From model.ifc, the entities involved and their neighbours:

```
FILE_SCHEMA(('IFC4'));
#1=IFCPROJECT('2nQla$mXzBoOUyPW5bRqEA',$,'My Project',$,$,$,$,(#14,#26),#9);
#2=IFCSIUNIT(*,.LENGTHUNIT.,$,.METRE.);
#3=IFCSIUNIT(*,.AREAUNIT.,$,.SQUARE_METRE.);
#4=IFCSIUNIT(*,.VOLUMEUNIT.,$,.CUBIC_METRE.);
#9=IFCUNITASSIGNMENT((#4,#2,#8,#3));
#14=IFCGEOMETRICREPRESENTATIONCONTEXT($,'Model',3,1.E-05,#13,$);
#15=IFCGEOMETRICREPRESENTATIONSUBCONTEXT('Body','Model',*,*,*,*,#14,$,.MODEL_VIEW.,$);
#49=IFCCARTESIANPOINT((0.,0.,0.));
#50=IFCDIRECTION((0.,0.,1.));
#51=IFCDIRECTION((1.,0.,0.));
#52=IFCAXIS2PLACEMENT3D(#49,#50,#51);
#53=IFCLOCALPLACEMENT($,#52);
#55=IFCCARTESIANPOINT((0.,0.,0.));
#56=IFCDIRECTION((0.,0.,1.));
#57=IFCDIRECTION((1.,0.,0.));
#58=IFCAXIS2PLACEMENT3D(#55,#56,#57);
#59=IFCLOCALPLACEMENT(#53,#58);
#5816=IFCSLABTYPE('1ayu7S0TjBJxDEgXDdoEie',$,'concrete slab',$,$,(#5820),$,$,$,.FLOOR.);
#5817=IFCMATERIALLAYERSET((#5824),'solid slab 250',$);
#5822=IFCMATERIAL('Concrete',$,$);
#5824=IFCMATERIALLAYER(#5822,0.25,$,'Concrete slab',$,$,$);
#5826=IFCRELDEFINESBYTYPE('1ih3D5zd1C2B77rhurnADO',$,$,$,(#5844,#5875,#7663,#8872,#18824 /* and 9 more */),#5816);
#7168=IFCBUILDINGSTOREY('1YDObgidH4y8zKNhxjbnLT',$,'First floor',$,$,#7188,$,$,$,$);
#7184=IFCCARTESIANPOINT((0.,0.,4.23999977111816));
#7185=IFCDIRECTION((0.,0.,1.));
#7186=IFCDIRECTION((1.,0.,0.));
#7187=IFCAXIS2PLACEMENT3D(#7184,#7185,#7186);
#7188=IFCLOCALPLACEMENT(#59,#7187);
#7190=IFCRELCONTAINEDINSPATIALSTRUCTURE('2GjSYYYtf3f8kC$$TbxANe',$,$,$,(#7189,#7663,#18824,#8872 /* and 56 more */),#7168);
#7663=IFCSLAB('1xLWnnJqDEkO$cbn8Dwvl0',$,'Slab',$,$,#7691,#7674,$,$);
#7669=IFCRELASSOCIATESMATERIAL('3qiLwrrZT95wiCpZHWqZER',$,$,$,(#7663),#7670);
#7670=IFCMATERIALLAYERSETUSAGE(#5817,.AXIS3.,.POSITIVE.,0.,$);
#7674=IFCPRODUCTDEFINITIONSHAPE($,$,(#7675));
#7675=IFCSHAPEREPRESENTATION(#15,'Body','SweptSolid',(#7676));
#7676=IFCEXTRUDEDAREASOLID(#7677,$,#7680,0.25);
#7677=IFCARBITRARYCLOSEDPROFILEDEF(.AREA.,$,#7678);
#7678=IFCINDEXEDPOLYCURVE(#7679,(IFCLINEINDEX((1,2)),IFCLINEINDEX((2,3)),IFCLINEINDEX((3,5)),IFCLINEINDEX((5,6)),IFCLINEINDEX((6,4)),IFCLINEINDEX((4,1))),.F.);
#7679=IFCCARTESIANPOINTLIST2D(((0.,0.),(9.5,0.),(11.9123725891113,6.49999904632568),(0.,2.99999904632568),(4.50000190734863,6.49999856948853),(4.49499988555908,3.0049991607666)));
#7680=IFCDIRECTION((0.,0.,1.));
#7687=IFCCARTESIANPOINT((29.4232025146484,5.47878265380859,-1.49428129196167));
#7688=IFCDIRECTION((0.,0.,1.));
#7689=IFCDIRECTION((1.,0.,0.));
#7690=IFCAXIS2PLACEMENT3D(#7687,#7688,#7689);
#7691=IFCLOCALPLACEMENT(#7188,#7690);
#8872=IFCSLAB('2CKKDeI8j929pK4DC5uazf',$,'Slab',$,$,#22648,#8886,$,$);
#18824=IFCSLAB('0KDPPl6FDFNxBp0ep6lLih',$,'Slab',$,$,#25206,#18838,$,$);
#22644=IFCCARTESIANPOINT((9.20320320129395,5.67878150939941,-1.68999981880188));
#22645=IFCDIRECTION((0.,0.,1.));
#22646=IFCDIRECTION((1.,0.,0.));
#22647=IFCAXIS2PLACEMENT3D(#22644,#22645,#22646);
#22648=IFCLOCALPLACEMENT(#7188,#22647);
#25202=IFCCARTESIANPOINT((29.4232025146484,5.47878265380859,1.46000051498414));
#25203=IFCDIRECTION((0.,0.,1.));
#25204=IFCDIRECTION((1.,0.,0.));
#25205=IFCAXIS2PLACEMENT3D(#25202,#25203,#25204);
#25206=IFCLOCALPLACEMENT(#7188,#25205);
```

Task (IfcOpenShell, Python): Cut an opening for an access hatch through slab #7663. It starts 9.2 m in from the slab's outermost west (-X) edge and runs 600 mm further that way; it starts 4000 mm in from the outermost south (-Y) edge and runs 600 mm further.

```python
import numpy as np
import ifcopenshell
import ifcopenshell.api.feature
import ifcopenshell.api.geometry
import ifcopenshell.api.root
import ifcopenshell.geom
import ifcopenshell.util.placement
import ifcopenshell.util.representation
import ifcopenshell.util.shape
import ifcopenshell.util.unit

model = ifcopenshell.open("model.ifc")
unit_scale = ifcopenshell.util.unit.calculate_unit_scale(model)
settings = ifcopenshell.geom.settings()


def volume(element):
    """Net volume in cubic metres, openings subtracted."""
    shape = ifcopenshell.geom.create_shape(settings, element)
    return ifcopenshell.util.shape.get_volume(shape.geometry)


slab = model.by_guid("1xLWnnJqDEkO$cbn8Dwvl0")
before = volume(slab)

# Extent in the slab's own axes, in metres. The edges named are its -X and -Y sides.
slab_shape = ifcopenshell.geom.create_shape(settings, slab)
vertices = ifcopenshell.util.shape.get_vertices(slab_shape.geometry)
x_min, y_min, bottom = vertices.min(axis=0)
top = vertices[:, 2].max()

opening = ifcopenshell.api.root.create_entity(model, ifc_class="IfcOpeningElement", name="Access hatch opening", predefined_type="OPENING")
context = ifcopenshell.util.representation.get_context(model, "Model", "Body", "MODEL_VIEW")
width, depth = 0.6, 0.6
outline = [(0.0, 0.0), (width, 0.0), (width, depth), (0.0, depth), (0.0, 0.0)]
# Overshoot both faces by 50 mm so the cut is clean.
shape = ifcopenshell.api.geometry.add_slab_representation(
    model, context=context, depth=top - bottom + 0.1, polyline=outline
)
ifcopenshell.api.geometry.assign_representation(model, product=opening, representation=shape)

matrix = ifcopenshell.util.placement.get_local_placement(slab.ObjectPlacement)
matrix[:, 3] = matrix @ np.append(np.array([x_min + 9.2, y_min + 4, bottom - 0.05]) / unit_scale, 1.0)
ifcopenshell.api.geometry.edit_object_placement(model, product=opening, matrix=matrix, is_si=False)
ifcopenshell.api.feature.add_feature(model, feature=opening, element=slab)

after = volume(slab)

print(f"slab volume {before:.3f} -> {after:.3f} m3")

model.write("model_rev.ifc")
```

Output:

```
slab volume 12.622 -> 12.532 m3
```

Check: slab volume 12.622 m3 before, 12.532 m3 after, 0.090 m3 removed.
